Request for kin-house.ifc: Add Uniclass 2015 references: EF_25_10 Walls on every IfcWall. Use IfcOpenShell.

First a look at what the model holds.

```python
import ifcopenshell

model = ifcopenshell.open("kin-house.ifc")
print(model.schema)
print("classifications:", [c.Name for c in model.by_type("IfcClassification")])
for ifc_class in ("IfcDoor", "IfcRoof", "IfcStair", "IfcWall", "IfcWindow"):
    print(ifc_class, len(model.by_type(ifc_class)))
```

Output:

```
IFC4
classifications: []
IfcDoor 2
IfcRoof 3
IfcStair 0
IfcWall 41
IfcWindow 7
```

```python
import ifcopenshell
import ifcopenshell.api.classification

model = ifcopenshell.open("kin-house.ifc")

system = ifcopenshell.api.classification.add_classification(model, classification="Uniclass 2015")

codes = {
    "IfcWall": ("EF_25_10", "Walls"),
}
for ifc_class, (code, name) in codes.items():
    products = model.by_type(ifc_class)
    ifcopenshell.api.classification.add_reference(
        model, products=products, classification=system, identification=code, name=name
    )
    print(code, len(products))

model.write("kin-house_rev.ifc")
```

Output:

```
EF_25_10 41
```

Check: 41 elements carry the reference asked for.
